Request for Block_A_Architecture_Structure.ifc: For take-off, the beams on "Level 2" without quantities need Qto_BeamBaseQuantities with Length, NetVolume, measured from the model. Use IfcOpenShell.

First a look at what the model holds.

```python
import ifcopenshell
import ifcopenshell.util.element
import ifcopenshell.util.unit

model = ifcopenshell.open("Block_A_Architecture_Structure.ifc")
print(model.schema)
for unit_type in ("LENGTHUNIT", "AREAUNIT", "VOLUMEUNIT"):
    print(unit_type, ifcopenshell.util.unit.calculate_unit_scale(model, unit_type))
storey = next(s for s in model.by_type("IfcBuildingStorey") if s.Name == "Level 2")
beams = [e for e in ifcopenshell.util.element.get_decomposition(storey) if e.is_a("IfcBeam")]
for e in sorted(beams, key=lambda e: e.id()):
    print(e.id(), e.is_a(), e.Name, list(ifcopenshell.util.element.get_psets(e, qtos_only=True)), sep=" | ")
```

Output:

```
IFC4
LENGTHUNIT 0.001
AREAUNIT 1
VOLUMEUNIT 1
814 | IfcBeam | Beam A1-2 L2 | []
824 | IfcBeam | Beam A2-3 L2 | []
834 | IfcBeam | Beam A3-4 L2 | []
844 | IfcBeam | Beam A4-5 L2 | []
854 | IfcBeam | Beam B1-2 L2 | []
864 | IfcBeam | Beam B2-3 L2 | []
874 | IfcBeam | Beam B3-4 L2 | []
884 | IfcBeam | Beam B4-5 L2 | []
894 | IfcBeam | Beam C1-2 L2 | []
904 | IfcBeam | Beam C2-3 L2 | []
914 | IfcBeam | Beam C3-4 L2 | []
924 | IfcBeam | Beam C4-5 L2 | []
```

```python
import ifcopenshell
import ifcopenshell.api.pset
import ifcopenshell.geom
import ifcopenshell.util.element
import ifcopenshell.util.shape
import ifcopenshell.util.unit

model = ifcopenshell.open("Block_A_Architecture_Structure.ifc")
unit_scale = ifcopenshell.util.unit.calculate_unit_scale(model)
volume_scale = ifcopenshell.util.unit.calculate_unit_scale(model, "VOLUMEUNIT")
settings = ifcopenshell.geom.settings()

storey = next(s for s in model.by_type("IfcBuildingStorey") if s.Name == "Level 2")
beams = [e for e in ifcopenshell.util.element.get_decomposition(storey) if e.is_a("IfcBeam")]

for e in sorted(beams, key=lambda e: e.id()):
    if ifcopenshell.util.element.get_psets(e, qtos_only=True, should_inherit=False):
        continue
    # Geometry comes back in metres, in the element's own axes.
    shape = ifcopenshell.geom.create_shape(settings, e)
    values = {
        "Length": ifcopenshell.util.shape.get_max_xyz(shape.geometry) / unit_scale,
        "NetVolume": ifcopenshell.util.shape.get_volume(shape.geometry) / volume_scale,
    }
    qto = ifcopenshell.api.pset.add_qto(model, product=e, name="Qto_BeamBaseQuantities")
    ifcopenshell.api.pset.edit_qto(model, qto=qto, properties=values)
    print(e.id(), {k: round(v, 3) for k, v in values.items()})

model.write("Block_A_Architecture_Structure-out.ifc")
```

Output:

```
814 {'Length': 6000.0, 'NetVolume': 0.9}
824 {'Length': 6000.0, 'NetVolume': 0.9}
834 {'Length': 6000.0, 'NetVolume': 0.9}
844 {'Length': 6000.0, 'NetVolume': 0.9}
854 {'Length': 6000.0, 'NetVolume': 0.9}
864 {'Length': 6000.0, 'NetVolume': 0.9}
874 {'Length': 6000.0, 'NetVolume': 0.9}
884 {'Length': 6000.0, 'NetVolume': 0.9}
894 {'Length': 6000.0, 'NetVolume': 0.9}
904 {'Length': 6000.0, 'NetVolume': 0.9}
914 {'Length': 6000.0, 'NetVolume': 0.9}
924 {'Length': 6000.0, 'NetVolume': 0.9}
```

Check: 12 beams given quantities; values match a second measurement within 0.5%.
